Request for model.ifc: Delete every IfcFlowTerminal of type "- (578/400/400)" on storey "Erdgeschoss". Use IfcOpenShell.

First a look at what the model holds.

```python
import ifcopenshell
import ifcopenshell.util.element

model = ifcopenshell.open("model.ifc")
print(model.schema)
storey = next(s for s in model.by_type("IfcBuildingStorey") if s.Name == "Erdgeschoss")
terminals = [e for e in ifcopenshell.util.element.get_decomposition(storey) if e.is_a("IfcFlowTerminal")]
seen = {}
for e in terminals:
    element_type = ifcopenshell.util.element.get_type(e)
    name = element_type.Name if element_type not in (None, e) else None
    seen[name] = seen.get(name, 0) + 1
for name, count in sorted(seen.items(), key=str):
    print(count, "x", name)
```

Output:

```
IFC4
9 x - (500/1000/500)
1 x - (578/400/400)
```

```python
import ifcopenshell
import ifcopenshell.api.root
import ifcopenshell.util.element

model = ifcopenshell.open("model.ifc")

storey = next(s for s in model.by_type("IfcBuildingStorey") if s.Name == "Erdgeschoss")
terminals = [e for e in ifcopenshell.util.element.get_decomposition(storey) if e.is_a("IfcFlowTerminal")]
targets = [e for e in terminals if (t := ifcopenshell.util.element.get_type(e)) not in (None, e) and t.Name == "- (578/400/400)"]

for e in targets:
    ifcopenshell.api.root.remove_product(model, product=e)
print(len(targets), "removed")

model.write("model_updated.ifc")
```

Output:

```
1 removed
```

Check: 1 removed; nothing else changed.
